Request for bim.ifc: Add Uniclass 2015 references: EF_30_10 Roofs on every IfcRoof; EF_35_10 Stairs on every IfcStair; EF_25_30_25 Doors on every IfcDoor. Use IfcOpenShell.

First a look at what the model holds.

```python
import ifcopenshell

model = ifcopenshell.open("bim.ifc")
print(model.schema)
print("classifications:", [c.Name for c in model.by_type("IfcClassification")])
for ifc_class in ("IfcDoor", "IfcRoof", "IfcStair", "IfcWall", "IfcWindow"):
    print(ifc_class, len(model.by_type(ifc_class)))
```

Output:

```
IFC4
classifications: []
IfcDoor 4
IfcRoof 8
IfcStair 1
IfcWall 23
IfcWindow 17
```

```python
import ifcopenshell
import ifcopenshell.api.classification

model = ifcopenshell.open("bim.ifc")

system = ifcopenshell.api.classification.add_classification(model, classification="Uniclass 2015")

codes = {
    "IfcRoof": ("EF_30_10", "Roofs"),
    "IfcStair": ("EF_35_10", "Stairs"),
    "IfcDoor": ("EF_25_30_25", "Doors"),
}
for ifc_class, (code, name) in codes.items():
    products = model.by_type(ifc_class)
    ifcopenshell.api.classification.add_reference(
        model, products=products, classification=system, identification=code, name=name
    )
    print(code, len(products))

model.write("bim_rev.ifc")
```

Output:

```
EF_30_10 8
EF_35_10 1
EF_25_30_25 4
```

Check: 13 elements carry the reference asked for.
